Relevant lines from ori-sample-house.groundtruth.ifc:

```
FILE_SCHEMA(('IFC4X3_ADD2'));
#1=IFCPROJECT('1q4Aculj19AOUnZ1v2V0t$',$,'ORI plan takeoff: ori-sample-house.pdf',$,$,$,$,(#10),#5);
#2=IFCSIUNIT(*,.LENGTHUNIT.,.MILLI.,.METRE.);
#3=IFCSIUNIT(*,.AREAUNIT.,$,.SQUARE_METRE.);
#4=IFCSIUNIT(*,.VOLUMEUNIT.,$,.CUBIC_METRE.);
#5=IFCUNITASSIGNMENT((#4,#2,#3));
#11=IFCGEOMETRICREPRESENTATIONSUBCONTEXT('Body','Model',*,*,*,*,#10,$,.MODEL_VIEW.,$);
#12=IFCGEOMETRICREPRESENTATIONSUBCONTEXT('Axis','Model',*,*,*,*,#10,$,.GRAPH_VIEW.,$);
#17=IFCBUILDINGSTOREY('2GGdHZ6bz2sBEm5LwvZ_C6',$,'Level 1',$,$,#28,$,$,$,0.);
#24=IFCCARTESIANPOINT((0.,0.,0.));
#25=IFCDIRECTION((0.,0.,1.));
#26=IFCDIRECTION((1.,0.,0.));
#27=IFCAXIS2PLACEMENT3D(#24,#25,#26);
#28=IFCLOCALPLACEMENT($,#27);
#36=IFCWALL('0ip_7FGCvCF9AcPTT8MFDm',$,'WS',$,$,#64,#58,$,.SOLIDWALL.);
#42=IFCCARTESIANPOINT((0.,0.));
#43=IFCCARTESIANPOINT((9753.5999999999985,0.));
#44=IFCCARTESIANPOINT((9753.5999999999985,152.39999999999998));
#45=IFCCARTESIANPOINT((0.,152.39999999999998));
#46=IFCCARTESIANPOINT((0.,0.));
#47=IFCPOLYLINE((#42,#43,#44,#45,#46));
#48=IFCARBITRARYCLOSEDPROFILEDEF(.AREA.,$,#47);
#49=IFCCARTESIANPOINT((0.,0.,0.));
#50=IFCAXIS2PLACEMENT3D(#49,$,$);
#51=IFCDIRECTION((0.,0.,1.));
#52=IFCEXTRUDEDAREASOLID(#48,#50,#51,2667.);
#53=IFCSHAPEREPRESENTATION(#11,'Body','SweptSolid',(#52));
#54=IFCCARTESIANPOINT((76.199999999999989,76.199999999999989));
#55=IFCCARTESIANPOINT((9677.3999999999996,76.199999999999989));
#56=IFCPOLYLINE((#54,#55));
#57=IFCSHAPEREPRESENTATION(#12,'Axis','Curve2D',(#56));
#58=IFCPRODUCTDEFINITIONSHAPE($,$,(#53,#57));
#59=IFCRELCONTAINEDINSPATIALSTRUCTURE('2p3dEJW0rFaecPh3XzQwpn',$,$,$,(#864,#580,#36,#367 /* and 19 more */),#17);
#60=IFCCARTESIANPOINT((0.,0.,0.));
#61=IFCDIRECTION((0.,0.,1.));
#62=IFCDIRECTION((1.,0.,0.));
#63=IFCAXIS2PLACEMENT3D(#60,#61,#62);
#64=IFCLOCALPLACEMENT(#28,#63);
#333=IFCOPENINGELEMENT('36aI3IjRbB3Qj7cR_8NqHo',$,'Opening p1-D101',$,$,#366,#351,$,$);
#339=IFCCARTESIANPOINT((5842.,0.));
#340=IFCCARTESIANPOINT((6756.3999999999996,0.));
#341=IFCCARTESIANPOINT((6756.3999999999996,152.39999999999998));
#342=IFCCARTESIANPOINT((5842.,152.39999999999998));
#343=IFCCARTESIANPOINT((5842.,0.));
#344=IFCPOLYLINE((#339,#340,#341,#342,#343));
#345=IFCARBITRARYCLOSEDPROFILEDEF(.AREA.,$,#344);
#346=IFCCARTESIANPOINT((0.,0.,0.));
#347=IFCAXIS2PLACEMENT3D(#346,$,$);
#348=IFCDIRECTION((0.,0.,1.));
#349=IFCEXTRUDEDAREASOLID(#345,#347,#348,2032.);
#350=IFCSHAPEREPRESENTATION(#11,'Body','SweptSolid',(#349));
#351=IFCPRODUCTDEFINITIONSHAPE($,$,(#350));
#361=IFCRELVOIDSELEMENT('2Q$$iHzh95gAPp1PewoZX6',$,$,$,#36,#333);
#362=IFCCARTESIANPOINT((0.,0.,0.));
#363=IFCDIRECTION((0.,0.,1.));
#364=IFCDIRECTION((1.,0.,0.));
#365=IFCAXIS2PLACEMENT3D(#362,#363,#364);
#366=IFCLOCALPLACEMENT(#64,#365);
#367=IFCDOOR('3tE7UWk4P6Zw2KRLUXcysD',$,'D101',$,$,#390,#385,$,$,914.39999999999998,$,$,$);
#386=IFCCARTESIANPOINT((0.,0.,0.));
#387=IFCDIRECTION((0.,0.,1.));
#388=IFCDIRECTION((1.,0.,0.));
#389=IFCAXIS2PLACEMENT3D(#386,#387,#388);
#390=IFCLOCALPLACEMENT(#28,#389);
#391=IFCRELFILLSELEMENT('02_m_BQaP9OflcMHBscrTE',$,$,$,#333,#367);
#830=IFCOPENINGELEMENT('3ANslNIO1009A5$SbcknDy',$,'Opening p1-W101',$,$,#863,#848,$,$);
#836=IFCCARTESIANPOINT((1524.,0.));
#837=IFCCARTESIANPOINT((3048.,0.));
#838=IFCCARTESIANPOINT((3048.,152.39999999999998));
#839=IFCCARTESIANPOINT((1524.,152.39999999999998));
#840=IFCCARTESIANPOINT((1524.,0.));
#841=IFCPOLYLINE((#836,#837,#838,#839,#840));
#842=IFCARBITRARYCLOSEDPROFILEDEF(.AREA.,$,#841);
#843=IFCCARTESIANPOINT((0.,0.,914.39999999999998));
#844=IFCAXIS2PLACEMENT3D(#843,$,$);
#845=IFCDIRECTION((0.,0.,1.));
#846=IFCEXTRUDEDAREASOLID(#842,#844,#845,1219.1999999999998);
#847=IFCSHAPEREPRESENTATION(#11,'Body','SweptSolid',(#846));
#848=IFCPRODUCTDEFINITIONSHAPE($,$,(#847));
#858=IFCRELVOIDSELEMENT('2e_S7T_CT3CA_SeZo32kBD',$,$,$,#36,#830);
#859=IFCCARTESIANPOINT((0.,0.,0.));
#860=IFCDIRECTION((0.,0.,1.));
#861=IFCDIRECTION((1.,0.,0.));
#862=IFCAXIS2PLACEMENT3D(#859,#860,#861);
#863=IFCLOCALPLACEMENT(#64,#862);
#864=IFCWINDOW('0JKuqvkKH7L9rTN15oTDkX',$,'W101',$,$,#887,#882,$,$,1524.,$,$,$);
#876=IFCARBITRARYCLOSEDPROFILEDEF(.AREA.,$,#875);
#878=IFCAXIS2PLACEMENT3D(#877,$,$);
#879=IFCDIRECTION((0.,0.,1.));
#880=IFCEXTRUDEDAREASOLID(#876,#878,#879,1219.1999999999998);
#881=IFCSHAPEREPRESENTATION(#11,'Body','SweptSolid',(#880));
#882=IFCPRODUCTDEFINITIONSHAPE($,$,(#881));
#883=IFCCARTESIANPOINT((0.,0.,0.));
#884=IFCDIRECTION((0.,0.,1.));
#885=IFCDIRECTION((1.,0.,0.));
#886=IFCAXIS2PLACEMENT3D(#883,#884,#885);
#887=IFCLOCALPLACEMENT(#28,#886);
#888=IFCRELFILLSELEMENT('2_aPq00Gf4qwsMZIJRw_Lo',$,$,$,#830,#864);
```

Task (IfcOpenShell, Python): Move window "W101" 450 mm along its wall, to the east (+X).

```python
import ifcopenshell
import ifcopenshell.api.geometry
import ifcopenshell.util.placement
import ifcopenshell.util.unit

model = ifcopenshell.open("ori-sample-house.groundtruth.ifc")
unit_scale = ifcopenshell.util.unit.calculate_unit_scale(model)

window = model.by_guid("0JKuqvkKH7L9rTN15oTDkX")
opening = window.FillsVoids[0].RelatingOpeningElement
wall = opening.VoidsElements[0].RelatingBuildingElement

wall_matrix = ifcopenshell.util.placement.get_local_placement(wall.ObjectPlacement)
shift = wall_matrix[:3, 0] * 0.45 / unit_scale
before = ifcopenshell.util.placement.get_local_placement(window.ObjectPlacement)[:3, 3].copy()

# The window is not placed relative to its opening, so move both.
for product in (opening, window):
    matrix = ifcopenshell.util.placement.get_local_placement(product.ObjectPlacement)
    matrix[:3, 3] += shift
    ifcopenshell.api.geometry.edit_object_placement(model, product=product, matrix=matrix, is_si=False)

after = ifcopenshell.util.placement.get_local_placement(window.ObjectPlacement)[:3, 3]
print("window moved by", (after - before).round(3) + 0.0)

model.write("ori-sample-house.groundtruth_v2.ifc")
```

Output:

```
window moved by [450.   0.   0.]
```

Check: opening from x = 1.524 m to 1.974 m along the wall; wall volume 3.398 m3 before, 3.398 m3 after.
